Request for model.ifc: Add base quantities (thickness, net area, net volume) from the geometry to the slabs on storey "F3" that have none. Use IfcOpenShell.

First a look at what the model holds.

```python
import ifcopenshell
import ifcopenshell.util.element
import ifcopenshell.util.unit

model = ifcopenshell.open("model.ifc")
print(model.schema)
for unit_type in ("LENGTHUNIT", "AREAUNIT", "VOLUMEUNIT"):
    print(unit_type, ifcopenshell.util.unit.calculate_unit_scale(model, unit_type))
storey = next(s for s in model.by_type("IfcBuildingStorey") if s.Name == "F3")
slabs = [e for e in ifcopenshell.util.element.get_decomposition(storey) if e.is_a("IfcSlab")]
for e in sorted(slabs, key=lambda e: e.id()):
    print(e.id(), e.is_a(), e.Name, list(ifcopenshell.util.element.get_psets(e, qtos_only=True)), sep=" | ")
```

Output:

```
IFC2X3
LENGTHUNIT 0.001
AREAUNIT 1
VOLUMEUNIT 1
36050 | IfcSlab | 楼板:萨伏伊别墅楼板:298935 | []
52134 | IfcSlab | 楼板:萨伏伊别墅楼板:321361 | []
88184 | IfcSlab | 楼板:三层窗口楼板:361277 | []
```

```python
import ifcopenshell
import ifcopenshell.api.pset
import ifcopenshell.geom
import ifcopenshell.util.element
import ifcopenshell.util.shape
import ifcopenshell.util.unit

model = ifcopenshell.open("model.ifc")
unit_scale = ifcopenshell.util.unit.calculate_unit_scale(model)
area_scale = ifcopenshell.util.unit.calculate_unit_scale(model, "AREAUNIT")
volume_scale = ifcopenshell.util.unit.calculate_unit_scale(model, "VOLUMEUNIT")
settings = ifcopenshell.geom.settings()

storey = next(s for s in model.by_type("IfcBuildingStorey") if s.Name == "F3")
slabs = [e for e in ifcopenshell.util.element.get_decomposition(storey) if e.is_a("IfcSlab")]

for e in sorted(slabs, key=lambda e: e.id()):
    if ifcopenshell.util.element.get_psets(e, qtos_only=True, should_inherit=False):
        continue
    # Geometry comes back in metres, in the element's own axes.
    shape = ifcopenshell.geom.create_shape(settings, e)
    values = {
        "Width": ifcopenshell.util.shape.get_z(shape.geometry) / unit_scale,
        "NetArea": ifcopenshell.util.shape.get_footprint_area(shape.geometry) / area_scale,
        "NetVolume": ifcopenshell.util.shape.get_volume(shape.geometry) / volume_scale,
    }
    qto = ifcopenshell.api.pset.add_qto(model, product=e, name="BaseQuantities")
    ifcopenshell.api.pset.edit_qto(model, qto=qto, properties=values)
    print(e.id(), {k: round(v, 3) for k, v in values.items()})

model.write("model_edited.ifc")
```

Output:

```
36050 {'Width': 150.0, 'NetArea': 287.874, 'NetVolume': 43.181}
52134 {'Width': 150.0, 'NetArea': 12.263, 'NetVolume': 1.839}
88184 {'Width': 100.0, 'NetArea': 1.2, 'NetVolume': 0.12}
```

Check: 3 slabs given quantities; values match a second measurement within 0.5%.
